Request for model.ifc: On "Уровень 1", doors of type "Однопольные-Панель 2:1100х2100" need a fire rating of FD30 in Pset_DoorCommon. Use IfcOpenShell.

First a look at what the model holds.

```python
import ifcopenshell
import ifcopenshell.util.element

model = ifcopenshell.open("model.ifc")
print(model.schema)
storey = next(s for s in model.by_type("IfcBuildingStorey") if s.Name == "Уровень 1")
doors = [e for e in ifcopenshell.util.element.get_decomposition(storey) if e.is_a("IfcDoor")]
seen = {}
for e in doors:
    element_type = ifcopenshell.util.element.get_type(e)
    key = (element_type.Name if element_type != e and element_type else None, ifcopenshell.util.element.get_pset(e, "Pset_DoorCommon", "FireRating"))
    seen[key] = seen.get(key, 0) + 1
for (name, value), count in sorted(seen.items(), key=str):
    print(count, "x", name, "|", value)
```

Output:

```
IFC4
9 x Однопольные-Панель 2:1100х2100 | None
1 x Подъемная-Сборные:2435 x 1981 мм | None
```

```python
import ifcopenshell
import ifcopenshell.api.pset
import ifcopenshell.util.element

model = ifcopenshell.open("model.ifc")

storey = next(s for s in model.by_type("IfcBuildingStorey") if s.Name == "Уровень 1")
doors = [e for e in ifcopenshell.util.element.get_decomposition(storey) if e.is_a("IfcDoor")]

count = 0
for e in doors:
    element_type = ifcopenshell.util.element.get_type(e)
    if element_type in (None, e) or element_type.Name != "Однопольные-Панель 2:1100х2100":
        continue
    # add_pset returns the element's existing set when there is one.
    pset = ifcopenshell.api.pset.add_pset(model, product=e, name="Pset_DoorCommon")
    ifcopenshell.api.pset.edit_pset(model, pset=pset, properties={"FireRating": "FD30"})
    count += 1

print(count, "doors updated")

model.write("model_updated.ifc")
```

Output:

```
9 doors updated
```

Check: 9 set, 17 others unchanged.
